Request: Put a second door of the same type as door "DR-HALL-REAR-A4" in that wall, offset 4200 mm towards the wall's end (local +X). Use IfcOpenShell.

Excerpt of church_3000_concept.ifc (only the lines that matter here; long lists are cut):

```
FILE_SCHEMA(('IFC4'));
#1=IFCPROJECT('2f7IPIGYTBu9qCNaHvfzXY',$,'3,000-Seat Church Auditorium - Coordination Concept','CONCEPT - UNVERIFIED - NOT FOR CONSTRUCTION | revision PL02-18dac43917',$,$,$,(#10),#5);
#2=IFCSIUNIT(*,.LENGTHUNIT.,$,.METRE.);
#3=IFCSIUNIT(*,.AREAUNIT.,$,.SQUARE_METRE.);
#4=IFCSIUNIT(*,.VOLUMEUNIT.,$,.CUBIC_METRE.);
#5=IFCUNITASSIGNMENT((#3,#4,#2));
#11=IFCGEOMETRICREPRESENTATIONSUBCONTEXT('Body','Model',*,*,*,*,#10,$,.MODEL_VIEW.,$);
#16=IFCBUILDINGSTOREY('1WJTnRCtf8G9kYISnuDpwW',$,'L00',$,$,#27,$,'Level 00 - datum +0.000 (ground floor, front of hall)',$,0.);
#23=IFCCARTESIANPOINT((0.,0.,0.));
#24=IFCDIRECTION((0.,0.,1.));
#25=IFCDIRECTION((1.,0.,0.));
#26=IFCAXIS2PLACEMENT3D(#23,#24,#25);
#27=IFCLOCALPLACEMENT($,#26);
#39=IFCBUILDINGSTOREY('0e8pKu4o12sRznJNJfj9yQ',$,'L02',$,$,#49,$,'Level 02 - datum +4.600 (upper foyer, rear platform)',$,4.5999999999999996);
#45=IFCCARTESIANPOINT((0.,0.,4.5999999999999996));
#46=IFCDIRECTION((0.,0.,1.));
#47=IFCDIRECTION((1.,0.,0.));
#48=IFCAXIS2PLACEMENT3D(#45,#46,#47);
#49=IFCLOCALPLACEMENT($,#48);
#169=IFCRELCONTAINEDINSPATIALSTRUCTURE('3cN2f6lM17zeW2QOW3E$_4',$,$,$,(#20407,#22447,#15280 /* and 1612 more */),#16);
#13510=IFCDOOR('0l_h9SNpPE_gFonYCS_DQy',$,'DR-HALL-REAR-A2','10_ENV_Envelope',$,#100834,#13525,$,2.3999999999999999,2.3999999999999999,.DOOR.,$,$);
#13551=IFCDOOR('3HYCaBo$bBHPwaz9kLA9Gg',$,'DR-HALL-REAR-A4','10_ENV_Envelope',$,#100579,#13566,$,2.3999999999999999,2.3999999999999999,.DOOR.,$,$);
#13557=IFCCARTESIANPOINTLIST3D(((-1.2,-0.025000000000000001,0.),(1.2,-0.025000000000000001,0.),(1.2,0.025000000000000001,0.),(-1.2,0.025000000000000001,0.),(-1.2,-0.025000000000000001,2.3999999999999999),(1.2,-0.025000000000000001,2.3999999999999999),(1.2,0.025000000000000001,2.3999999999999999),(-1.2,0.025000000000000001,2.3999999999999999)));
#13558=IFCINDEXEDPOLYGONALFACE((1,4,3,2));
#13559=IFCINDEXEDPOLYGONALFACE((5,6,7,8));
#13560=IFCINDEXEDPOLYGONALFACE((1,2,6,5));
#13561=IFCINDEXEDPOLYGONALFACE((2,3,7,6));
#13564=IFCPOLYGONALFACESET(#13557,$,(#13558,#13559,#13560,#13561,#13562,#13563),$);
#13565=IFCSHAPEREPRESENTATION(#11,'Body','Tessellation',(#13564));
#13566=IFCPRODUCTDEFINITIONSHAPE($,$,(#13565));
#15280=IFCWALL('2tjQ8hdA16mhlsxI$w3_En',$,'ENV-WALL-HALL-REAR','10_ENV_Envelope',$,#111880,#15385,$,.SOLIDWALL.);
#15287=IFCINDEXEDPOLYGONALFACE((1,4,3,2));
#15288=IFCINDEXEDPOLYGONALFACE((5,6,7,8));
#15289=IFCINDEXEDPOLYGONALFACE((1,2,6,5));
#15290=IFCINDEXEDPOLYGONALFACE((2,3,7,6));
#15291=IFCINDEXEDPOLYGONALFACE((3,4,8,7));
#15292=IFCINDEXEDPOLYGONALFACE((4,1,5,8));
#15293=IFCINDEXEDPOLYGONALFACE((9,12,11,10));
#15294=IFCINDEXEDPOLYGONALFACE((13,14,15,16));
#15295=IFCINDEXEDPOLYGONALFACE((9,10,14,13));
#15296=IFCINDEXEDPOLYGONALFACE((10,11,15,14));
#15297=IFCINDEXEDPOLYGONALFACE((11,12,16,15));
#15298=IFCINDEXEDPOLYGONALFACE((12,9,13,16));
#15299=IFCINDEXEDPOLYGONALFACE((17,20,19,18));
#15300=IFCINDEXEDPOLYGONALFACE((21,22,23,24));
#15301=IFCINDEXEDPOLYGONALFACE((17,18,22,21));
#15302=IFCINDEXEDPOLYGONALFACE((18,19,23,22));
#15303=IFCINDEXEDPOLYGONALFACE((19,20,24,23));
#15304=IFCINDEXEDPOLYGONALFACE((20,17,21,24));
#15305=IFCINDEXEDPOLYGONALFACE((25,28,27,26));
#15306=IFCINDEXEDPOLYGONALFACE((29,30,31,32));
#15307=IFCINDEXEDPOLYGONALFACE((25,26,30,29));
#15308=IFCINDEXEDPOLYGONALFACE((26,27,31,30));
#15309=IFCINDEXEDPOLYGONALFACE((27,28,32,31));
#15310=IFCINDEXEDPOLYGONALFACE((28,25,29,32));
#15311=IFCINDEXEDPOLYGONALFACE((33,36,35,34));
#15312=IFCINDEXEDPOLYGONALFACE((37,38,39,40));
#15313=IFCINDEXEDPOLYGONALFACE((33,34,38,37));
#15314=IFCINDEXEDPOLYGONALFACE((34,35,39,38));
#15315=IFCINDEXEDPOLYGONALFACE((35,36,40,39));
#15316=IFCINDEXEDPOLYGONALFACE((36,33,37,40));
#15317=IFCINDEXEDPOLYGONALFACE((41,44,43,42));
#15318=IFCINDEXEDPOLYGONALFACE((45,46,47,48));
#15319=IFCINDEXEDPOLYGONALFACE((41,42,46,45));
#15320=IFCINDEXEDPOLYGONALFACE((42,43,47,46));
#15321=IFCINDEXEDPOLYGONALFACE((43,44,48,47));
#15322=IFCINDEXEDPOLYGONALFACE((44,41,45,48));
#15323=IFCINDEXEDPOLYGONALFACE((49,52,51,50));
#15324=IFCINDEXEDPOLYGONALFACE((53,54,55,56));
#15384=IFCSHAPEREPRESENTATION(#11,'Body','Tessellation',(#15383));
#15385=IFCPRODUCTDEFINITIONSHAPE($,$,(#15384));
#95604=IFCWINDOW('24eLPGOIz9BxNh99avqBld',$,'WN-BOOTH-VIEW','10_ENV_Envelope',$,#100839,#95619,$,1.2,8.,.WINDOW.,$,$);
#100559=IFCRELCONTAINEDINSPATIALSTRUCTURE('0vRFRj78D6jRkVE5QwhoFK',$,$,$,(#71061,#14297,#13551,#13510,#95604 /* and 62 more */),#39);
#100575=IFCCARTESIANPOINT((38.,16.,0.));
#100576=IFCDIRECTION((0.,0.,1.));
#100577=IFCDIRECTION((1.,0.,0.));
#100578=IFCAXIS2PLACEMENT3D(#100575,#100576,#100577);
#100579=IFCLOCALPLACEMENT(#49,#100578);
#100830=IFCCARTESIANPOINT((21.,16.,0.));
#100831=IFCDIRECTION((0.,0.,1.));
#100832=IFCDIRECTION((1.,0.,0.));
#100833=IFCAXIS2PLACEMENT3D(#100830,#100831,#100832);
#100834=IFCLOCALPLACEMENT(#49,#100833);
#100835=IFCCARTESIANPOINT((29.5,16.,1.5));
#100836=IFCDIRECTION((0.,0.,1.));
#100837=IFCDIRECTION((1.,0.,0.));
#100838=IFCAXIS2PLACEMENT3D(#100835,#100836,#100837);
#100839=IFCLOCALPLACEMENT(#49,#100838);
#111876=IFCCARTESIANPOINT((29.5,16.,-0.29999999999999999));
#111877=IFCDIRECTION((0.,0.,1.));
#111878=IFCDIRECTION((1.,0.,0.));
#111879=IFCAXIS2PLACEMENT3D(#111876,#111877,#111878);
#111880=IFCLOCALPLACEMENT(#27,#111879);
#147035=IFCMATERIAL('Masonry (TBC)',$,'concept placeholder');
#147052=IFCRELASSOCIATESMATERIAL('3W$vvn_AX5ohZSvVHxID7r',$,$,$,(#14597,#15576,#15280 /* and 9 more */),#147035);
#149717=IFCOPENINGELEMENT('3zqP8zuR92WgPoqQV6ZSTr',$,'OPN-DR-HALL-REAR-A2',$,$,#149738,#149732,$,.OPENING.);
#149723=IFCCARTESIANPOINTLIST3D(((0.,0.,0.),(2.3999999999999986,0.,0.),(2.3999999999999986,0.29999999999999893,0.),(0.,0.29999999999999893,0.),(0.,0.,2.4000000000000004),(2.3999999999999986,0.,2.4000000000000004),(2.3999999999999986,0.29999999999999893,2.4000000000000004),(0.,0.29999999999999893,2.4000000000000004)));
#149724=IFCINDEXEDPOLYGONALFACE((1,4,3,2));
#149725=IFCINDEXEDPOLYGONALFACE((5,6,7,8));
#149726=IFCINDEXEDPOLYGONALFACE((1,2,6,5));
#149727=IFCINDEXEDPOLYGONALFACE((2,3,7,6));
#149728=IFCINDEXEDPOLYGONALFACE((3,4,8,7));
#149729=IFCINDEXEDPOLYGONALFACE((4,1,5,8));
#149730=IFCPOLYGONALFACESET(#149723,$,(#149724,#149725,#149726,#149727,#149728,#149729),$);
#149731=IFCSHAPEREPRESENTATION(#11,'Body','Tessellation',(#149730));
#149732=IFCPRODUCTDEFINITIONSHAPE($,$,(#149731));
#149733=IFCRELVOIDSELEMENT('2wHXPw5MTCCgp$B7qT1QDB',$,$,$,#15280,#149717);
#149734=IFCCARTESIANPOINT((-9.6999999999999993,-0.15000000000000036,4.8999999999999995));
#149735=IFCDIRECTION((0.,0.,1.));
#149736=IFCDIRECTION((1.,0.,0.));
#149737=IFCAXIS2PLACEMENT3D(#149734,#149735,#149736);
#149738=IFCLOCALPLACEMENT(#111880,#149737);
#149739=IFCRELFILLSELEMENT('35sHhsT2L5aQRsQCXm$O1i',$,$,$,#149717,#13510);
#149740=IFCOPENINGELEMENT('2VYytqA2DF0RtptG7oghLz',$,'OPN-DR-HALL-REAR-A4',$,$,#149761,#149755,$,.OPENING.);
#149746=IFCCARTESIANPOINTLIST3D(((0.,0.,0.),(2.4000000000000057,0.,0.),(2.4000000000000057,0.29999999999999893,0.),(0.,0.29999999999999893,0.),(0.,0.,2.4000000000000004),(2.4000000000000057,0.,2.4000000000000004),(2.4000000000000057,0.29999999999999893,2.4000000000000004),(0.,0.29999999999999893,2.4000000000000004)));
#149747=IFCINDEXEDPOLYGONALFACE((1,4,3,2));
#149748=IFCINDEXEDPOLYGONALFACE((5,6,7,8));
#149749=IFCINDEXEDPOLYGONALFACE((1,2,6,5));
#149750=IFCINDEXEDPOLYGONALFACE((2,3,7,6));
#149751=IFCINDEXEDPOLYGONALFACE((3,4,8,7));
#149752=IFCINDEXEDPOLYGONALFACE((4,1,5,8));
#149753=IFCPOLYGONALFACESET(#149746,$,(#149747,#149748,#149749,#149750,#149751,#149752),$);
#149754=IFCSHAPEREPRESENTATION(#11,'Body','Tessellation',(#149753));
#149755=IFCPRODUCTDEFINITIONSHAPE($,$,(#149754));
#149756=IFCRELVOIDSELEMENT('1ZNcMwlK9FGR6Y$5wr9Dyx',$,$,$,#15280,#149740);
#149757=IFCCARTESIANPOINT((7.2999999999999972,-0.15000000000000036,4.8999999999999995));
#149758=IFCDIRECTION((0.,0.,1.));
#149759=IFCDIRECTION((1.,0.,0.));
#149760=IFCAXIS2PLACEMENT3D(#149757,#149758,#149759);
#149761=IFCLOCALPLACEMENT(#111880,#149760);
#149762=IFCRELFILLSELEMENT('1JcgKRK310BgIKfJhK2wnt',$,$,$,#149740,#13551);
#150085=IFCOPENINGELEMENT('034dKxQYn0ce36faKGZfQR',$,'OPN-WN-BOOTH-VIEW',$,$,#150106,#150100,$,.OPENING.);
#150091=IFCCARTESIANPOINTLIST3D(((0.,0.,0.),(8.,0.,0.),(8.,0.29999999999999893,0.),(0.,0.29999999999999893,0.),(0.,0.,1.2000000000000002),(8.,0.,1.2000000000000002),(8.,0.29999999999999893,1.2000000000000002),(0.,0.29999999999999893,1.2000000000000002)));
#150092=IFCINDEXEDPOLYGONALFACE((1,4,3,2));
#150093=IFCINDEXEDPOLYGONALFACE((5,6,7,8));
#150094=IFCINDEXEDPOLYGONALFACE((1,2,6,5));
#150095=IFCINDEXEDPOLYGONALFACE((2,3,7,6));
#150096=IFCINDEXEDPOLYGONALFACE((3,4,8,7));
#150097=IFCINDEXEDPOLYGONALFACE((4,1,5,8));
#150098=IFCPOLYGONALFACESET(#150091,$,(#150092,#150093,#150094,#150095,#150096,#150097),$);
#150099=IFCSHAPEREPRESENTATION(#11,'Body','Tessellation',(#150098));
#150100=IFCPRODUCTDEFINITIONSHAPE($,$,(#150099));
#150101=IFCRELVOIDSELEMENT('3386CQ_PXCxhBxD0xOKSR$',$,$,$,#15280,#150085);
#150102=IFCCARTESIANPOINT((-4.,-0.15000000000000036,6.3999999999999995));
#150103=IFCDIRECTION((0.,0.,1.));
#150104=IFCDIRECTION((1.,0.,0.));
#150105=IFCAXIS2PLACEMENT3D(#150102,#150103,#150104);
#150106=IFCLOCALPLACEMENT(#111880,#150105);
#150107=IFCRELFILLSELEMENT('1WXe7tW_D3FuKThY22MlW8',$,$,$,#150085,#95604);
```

```python
import ifcopenshell
import ifcopenshell.api.feature
import ifcopenshell.api.geometry
import ifcopenshell.api.root
import ifcopenshell.geom
import ifcopenshell.util.element
import ifcopenshell.util.placement
import ifcopenshell.util.shape

model = ifcopenshell.open("church_3000_concept.ifc")
settings = ifcopenshell.geom.settings()


def volume(element):
    """Net volume in cubic metres, openings subtracted."""
    shape = ifcopenshell.geom.create_shape(settings, element)
    return ifcopenshell.util.shape.get_volume(shape.geometry)


door = model.by_guid("3HYCaBo$bBHPwaz9kLA9Gg")
opening = door.FillsVoids[0].RelatingOpeningElement
wall = opening.VoidsElements[0].RelatingBuildingElement
before = volume(wall)
shift = ifcopenshell.util.placement.get_local_placement(wall.ObjectPlacement)[:3, 0] * 4.2

# copy_class copies the void relationship, type, container and properties, but no geometry.
new_opening = ifcopenshell.api.root.copy_class(model, product=opening)
new_opening.Representation = ifcopenshell.util.element.copy_deep(
    model, opening.Representation, exclude=["IfcGeometricRepresentationContext", "IfcRepresentationMap"]
)
new_door = ifcopenshell.api.root.copy_class(model, product=door)
new_door.Representation = ifcopenshell.util.element.copy_deep(
    model, door.Representation, exclude=["IfcGeometricRepresentationContext", "IfcRepresentationMap"]
)
ifcopenshell.api.feature.add_filling(model, opening=new_opening, element=new_door)

for old, new in ((opening, new_opening), (door, new_door)):
    matrix = ifcopenshell.util.placement.get_local_placement(old.ObjectPlacement)
    matrix[:3, 3] += shift
    ifcopenshell.api.geometry.edit_object_placement(model, product=new, matrix=matrix, is_si=False)

after = volume(wall)

print(f"wall volume {before:.3f} -> {after:.3f} m3")

model.write("church_3000_concept_updated.ifc")
```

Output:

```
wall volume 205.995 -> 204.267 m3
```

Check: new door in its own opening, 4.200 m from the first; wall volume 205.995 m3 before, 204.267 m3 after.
